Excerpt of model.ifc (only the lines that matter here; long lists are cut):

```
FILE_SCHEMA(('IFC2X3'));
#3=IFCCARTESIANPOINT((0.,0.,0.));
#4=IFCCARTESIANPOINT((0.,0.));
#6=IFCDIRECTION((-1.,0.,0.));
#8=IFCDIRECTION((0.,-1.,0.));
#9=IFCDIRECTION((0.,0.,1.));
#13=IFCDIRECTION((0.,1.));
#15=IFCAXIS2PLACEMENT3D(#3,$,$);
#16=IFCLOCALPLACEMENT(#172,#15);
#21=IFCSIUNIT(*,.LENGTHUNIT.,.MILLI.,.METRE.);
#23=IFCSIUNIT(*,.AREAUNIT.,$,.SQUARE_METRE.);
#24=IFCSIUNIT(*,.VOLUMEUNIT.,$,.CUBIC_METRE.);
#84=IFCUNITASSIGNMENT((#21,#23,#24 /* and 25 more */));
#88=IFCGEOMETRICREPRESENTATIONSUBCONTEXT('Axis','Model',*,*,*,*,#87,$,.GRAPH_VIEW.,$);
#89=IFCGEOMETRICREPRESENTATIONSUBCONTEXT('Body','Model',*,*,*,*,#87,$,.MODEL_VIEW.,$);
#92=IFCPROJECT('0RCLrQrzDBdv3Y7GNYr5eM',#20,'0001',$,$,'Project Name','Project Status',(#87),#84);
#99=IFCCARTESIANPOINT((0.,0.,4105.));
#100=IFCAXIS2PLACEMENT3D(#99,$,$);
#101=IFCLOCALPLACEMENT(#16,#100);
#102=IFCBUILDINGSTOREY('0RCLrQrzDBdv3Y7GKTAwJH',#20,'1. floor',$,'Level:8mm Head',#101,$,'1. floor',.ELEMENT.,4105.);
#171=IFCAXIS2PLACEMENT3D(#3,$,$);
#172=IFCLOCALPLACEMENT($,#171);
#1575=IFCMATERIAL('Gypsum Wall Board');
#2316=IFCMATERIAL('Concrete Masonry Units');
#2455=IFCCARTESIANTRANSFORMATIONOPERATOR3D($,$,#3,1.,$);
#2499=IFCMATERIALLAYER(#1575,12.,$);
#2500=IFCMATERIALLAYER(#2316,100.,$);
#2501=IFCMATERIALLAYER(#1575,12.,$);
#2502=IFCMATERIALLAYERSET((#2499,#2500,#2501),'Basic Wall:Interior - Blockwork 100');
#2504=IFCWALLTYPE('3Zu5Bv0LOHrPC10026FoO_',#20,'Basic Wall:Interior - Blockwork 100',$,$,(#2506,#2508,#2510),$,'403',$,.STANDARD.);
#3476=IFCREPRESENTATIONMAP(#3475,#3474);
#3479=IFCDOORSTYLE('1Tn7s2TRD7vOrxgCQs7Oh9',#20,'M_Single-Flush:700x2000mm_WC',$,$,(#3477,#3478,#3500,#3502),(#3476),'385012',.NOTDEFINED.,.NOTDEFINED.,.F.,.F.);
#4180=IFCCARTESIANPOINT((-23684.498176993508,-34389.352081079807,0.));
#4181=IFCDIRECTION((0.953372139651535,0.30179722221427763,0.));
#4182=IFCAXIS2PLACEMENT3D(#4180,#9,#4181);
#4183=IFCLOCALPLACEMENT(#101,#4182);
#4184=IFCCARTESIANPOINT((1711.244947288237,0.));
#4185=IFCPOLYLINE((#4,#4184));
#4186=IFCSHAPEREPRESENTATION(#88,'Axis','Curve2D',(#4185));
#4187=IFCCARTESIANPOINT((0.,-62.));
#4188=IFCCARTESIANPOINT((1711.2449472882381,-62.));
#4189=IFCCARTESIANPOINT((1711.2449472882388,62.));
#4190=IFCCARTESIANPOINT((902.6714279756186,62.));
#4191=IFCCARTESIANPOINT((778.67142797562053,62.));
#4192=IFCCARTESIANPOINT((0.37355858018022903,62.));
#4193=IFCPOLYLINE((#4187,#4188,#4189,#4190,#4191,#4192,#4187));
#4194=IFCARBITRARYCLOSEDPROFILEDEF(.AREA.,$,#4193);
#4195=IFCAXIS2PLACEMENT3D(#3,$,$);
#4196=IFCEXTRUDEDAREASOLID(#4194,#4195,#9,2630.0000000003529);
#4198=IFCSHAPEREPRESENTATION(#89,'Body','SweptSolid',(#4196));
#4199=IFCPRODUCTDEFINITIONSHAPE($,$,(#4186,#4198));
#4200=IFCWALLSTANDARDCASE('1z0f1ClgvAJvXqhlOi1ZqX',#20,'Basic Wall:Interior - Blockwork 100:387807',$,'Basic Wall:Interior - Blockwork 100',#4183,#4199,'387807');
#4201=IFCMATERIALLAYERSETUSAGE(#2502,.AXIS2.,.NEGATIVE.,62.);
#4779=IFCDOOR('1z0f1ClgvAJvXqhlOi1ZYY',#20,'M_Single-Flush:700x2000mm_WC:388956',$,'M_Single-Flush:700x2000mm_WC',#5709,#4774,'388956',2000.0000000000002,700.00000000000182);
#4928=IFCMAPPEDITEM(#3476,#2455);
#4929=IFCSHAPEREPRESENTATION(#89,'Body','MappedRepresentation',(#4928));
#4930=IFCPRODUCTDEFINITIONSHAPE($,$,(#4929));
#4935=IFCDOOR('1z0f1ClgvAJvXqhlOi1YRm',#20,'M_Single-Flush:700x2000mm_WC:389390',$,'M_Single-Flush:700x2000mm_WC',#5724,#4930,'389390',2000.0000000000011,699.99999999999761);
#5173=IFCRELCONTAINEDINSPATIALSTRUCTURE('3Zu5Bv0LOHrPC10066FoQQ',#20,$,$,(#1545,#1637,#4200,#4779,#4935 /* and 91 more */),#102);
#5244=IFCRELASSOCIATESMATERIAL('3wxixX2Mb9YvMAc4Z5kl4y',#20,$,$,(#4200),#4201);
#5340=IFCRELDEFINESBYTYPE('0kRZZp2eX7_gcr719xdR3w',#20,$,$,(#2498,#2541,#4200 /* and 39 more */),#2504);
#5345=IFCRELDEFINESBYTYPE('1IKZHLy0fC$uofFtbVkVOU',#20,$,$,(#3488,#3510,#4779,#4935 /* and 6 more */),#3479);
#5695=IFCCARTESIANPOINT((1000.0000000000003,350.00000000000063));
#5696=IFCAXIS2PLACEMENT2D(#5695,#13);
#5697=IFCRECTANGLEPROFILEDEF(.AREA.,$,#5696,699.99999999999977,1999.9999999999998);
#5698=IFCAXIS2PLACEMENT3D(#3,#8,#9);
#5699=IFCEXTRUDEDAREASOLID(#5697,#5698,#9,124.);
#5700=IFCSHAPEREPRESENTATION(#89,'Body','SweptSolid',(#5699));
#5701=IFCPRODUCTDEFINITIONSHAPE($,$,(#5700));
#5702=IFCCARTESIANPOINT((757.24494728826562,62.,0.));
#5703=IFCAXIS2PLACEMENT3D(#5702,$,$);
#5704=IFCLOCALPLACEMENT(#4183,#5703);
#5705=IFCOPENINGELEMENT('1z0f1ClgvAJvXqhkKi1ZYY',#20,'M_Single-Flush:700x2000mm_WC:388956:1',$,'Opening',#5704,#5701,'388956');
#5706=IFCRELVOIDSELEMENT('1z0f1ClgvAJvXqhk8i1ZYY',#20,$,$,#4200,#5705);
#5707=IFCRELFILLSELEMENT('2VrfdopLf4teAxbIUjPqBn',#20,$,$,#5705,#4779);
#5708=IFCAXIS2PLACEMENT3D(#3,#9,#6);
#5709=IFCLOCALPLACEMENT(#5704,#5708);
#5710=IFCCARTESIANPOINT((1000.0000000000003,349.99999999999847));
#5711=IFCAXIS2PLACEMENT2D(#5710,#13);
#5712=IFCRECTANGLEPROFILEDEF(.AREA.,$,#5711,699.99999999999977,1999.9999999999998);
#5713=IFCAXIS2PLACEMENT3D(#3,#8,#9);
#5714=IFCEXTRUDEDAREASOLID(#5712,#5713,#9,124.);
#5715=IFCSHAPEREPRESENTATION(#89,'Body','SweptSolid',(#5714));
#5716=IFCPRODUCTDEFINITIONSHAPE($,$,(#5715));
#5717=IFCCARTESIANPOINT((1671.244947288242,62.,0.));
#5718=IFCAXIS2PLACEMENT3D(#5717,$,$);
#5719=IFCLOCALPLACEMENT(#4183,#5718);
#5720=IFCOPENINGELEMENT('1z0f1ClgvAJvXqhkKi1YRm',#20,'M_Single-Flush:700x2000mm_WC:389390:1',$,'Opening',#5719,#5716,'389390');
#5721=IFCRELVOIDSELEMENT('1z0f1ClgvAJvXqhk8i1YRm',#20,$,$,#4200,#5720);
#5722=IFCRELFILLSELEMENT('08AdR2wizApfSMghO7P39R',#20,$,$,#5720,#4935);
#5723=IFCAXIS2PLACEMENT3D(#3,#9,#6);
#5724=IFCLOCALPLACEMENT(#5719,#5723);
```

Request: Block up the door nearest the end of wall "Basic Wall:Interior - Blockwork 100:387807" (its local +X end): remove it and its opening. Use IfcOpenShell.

```python
import ifcopenshell
import ifcopenshell.api.feature
import ifcopenshell.api.root
import ifcopenshell.geom
import ifcopenshell.util.shape

model = ifcopenshell.open("model.ifc")
settings = ifcopenshell.geom.settings()


def volume(element):
    """Net volume in cubic metres, openings subtracted."""
    shape = ifcopenshell.geom.create_shape(settings, element)
    return ifcopenshell.util.shape.get_volume(shape.geometry)


door = model.by_id(4935)
opening = door.FillsVoids[0].RelatingOpeningElement
wall = opening.VoidsElements[0].RelatingBuildingElement
before = volume(wall)

ifcopenshell.api.root.remove_product(model, product=door)
ifcopenshell.api.feature.remove_feature(model, feature=opening)

after = volume(wall)

print(f"wall volume {before:.3f} -> {after:.3f} m3")

model.write("model_v2.ifc")
```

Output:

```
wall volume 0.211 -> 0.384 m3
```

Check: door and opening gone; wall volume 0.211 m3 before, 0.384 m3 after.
